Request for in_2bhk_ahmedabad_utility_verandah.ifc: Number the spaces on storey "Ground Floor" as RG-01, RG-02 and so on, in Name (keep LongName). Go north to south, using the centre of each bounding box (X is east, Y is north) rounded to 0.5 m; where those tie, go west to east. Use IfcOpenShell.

First a look at what the model holds.

```python
import ifcopenshell
import ifcopenshell.util.element
import ifcopenshell.util.placement

model = ifcopenshell.open("in_2bhk_ahmedabad_utility_verandah.ifc")
print(model.schema)
storey = next(s for s in model.by_type("IfcBuildingStorey") if s.Name == "Ground Floor")
spaces = [e for e in ifcopenshell.util.element.get_decomposition(storey) if e.is_a("IfcSpace")]
for e in sorted(spaces, key=lambda e: e.id()):
    origin = ifcopenshell.util.placement.get_local_placement(e.ObjectPlacement)[:3, 3]
    print(e.id(), e.Name, e.LongName, origin.round(2) + 0.0, sep=" | ")
```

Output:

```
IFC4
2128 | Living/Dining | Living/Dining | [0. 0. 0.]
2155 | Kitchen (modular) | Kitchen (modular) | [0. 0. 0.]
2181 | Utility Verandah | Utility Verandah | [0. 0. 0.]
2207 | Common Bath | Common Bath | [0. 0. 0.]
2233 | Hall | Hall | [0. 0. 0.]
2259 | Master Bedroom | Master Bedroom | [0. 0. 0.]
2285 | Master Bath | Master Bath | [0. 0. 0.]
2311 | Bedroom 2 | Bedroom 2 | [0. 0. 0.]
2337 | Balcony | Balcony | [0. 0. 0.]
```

```python
import ifcopenshell
import ifcopenshell.geom
import ifcopenshell.util.element
import ifcopenshell.util.shape

model = ifcopenshell.open("in_2bhk_ahmedabad_utility_verandah.ifc")
settings = ifcopenshell.geom.settings()
settings.set("use-world-coords", True)


def centre(element):
    shape = ifcopenshell.geom.create_shape(settings, element)
    return ifcopenshell.util.shape.get_bbox_centroid(shape.geometry)


storey = next(s for s in model.by_type("IfcBuildingStorey") if s.Name == "Ground Floor")
spaces = [e for e in ifcopenshell.util.element.get_decomposition(storey) if e.is_a("IfcSpace")]

# Insertion points can sit at a corner or the storey origin, so sort by the geometry (in metres).
centres = {e: centre(e) for e in spaces}
spaces.sort(key=lambda e: (-round(centres[e][1] / 0.5), centres[e][0]))

for i, e in enumerate(spaces, start=1):
    number = f"RG-{i:02d}"
    e.Name = number
    print(e.id(), number)

model.write("in_2bhk_ahmedabad_utility_verandah_edited.ifc")
```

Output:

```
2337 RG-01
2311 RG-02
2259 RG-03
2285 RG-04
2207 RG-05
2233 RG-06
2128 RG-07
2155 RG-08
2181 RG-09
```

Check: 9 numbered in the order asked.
